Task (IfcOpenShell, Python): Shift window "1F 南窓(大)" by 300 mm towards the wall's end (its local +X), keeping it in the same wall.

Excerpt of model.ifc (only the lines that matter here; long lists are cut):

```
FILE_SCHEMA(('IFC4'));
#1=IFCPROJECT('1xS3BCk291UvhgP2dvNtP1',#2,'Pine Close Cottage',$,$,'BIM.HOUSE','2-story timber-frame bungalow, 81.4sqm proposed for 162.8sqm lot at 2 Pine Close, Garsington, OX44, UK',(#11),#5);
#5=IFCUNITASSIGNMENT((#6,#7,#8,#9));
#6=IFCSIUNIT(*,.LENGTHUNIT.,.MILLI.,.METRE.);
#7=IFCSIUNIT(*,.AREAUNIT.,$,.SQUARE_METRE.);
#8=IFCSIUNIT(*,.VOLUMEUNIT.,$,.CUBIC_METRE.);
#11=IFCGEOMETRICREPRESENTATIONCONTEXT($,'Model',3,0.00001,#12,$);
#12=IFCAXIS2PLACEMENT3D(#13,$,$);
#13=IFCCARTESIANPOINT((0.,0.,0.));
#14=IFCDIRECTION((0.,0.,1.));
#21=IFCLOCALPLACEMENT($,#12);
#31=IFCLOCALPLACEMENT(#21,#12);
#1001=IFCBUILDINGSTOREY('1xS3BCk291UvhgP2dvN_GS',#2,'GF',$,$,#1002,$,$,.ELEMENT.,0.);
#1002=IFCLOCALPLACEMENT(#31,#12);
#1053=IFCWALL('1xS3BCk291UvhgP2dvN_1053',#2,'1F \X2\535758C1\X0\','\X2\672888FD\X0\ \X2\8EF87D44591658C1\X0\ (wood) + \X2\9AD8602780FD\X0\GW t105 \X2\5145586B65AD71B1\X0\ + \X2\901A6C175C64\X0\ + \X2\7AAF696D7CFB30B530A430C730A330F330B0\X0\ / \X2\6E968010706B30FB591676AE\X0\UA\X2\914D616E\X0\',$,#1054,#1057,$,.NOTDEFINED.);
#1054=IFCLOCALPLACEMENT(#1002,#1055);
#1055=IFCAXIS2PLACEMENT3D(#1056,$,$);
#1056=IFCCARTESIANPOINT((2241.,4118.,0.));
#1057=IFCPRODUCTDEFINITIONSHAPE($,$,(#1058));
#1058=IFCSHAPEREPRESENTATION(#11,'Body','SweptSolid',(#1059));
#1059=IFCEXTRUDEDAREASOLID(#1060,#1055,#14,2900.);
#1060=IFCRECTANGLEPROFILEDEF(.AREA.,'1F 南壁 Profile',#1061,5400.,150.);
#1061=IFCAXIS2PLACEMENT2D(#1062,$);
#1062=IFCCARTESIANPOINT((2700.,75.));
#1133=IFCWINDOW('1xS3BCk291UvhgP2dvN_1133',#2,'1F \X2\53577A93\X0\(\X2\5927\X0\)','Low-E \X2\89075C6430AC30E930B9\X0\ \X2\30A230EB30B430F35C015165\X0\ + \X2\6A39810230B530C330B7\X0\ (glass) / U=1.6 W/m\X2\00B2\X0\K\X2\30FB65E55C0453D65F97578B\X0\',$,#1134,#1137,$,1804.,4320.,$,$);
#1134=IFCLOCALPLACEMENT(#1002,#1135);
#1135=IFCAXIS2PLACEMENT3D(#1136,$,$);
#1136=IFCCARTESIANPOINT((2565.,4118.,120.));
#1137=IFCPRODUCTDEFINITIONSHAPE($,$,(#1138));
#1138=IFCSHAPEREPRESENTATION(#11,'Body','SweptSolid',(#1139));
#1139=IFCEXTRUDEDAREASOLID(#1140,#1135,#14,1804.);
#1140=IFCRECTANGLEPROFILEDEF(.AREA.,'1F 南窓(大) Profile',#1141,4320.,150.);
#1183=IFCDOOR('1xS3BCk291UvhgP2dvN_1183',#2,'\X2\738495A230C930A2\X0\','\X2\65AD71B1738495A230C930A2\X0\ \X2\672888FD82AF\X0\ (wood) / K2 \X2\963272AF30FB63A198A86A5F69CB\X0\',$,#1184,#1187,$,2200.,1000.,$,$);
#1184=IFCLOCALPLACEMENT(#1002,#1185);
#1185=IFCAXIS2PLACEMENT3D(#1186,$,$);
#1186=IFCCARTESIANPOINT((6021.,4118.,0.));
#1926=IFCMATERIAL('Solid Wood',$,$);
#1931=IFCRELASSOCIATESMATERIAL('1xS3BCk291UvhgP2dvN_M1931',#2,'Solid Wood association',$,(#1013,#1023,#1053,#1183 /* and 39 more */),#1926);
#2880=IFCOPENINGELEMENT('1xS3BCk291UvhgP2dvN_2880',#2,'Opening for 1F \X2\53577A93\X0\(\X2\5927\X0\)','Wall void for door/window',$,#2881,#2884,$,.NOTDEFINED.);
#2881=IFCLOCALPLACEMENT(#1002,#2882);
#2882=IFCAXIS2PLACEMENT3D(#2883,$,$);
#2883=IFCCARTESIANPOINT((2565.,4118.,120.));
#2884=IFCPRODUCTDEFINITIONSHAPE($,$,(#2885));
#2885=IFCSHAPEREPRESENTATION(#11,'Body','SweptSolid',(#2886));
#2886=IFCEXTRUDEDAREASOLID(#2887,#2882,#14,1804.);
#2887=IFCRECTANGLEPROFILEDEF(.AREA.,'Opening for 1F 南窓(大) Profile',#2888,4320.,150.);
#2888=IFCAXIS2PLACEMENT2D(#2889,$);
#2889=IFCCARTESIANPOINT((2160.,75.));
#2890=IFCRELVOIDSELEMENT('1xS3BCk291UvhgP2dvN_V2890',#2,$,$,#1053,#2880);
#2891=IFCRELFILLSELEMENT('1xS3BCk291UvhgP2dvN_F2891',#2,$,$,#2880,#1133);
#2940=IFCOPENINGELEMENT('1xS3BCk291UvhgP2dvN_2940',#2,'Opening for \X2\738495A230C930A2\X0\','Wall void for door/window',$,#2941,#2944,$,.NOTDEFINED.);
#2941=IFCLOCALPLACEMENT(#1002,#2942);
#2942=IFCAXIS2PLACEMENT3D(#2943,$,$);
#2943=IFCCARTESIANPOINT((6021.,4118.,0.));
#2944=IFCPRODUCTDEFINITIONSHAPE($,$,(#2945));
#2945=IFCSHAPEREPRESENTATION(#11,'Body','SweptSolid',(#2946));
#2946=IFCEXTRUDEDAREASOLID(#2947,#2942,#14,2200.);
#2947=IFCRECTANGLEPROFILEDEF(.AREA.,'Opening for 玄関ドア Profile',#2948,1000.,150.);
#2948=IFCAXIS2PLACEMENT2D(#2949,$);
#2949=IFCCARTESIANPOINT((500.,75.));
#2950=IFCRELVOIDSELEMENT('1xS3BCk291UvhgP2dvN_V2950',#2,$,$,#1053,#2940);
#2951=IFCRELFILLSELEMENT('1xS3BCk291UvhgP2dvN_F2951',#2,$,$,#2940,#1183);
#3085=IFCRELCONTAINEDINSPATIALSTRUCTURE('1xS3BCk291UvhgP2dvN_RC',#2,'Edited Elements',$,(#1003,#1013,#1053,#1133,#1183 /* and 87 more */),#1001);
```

```python
import ifcopenshell
import ifcopenshell.api.geometry
import ifcopenshell.util.placement

model = ifcopenshell.open("model.ifc")

window = model.by_guid("1xS3BCk291UvhgP2dvN_1133")
opening = window.FillsVoids[0].RelatingOpeningElement
wall = opening.VoidsElements[0].RelatingBuildingElement

wall_matrix = ifcopenshell.util.placement.get_local_placement(wall.ObjectPlacement)
shift = wall_matrix[:3, 0] * 300.0
before = ifcopenshell.util.placement.get_local_placement(window.ObjectPlacement)[:3, 3].copy()

# The window is not placed relative to its opening, so move both.
for product in (opening, window):
    matrix = ifcopenshell.util.placement.get_local_placement(product.ObjectPlacement)
    matrix[:3, 3] += shift
    ifcopenshell.api.geometry.edit_object_placement(model, product=product, matrix=matrix, is_si=False)

after = ifcopenshell.util.placement.get_local_placement(window.ObjectPlacement)[:3, 3]
print("window moved by", (after - before).round(3) + 0.0)

model.write("model_updated.ifc")
```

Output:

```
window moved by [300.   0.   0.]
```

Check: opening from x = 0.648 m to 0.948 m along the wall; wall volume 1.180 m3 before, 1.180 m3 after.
